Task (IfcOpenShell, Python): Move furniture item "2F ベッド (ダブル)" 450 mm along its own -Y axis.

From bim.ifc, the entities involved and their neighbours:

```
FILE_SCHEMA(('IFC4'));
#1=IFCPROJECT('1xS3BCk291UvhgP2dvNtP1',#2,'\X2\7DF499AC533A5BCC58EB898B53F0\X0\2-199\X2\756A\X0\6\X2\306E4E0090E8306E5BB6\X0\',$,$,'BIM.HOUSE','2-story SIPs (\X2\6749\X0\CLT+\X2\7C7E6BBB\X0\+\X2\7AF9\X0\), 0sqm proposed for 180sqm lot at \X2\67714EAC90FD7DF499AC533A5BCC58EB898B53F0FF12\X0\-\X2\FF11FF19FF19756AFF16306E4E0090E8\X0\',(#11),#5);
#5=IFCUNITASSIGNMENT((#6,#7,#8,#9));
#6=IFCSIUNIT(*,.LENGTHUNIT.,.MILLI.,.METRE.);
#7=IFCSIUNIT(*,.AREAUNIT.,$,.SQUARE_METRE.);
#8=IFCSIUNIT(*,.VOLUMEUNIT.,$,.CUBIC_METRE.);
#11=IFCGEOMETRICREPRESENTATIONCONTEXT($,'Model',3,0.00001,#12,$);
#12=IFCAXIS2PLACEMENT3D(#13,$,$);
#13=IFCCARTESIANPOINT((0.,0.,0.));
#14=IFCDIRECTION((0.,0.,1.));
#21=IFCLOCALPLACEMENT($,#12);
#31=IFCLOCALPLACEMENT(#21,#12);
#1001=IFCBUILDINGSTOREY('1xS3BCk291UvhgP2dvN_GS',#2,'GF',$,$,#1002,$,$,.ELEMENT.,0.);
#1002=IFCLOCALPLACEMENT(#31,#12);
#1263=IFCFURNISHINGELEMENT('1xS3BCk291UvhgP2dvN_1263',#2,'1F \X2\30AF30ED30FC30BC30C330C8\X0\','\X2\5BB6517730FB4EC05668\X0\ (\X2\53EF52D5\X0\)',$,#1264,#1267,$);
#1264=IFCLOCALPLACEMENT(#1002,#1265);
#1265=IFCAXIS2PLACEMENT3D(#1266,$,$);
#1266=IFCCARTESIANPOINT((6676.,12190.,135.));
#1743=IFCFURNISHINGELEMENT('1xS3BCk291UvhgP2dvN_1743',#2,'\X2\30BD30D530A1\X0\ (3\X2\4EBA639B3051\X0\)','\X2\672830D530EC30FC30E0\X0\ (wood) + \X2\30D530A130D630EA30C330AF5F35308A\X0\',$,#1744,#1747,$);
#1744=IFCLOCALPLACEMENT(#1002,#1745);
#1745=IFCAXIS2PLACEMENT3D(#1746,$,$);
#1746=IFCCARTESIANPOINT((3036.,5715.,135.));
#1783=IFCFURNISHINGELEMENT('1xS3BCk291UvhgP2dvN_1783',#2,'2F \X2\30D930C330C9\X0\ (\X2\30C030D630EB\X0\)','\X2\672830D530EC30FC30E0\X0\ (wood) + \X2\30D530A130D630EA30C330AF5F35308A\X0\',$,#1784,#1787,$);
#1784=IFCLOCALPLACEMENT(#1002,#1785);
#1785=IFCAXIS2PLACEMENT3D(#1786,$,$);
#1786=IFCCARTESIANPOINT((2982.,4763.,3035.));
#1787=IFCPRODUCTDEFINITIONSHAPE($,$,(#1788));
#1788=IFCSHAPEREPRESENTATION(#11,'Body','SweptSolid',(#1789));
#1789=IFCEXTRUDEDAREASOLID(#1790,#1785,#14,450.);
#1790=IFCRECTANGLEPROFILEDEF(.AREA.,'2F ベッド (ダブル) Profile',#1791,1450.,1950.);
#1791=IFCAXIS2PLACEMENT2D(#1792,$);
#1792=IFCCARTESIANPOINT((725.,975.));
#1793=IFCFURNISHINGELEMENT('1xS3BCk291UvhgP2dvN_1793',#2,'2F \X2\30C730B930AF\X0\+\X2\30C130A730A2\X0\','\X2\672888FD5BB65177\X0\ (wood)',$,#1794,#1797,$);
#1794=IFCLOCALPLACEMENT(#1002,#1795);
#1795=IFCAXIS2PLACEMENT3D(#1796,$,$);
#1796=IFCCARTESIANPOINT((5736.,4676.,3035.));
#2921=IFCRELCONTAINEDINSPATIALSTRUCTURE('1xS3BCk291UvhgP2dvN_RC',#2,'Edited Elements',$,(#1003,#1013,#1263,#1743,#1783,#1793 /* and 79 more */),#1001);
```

```python
import ifcopenshell
import ifcopenshell.api.geometry
import ifcopenshell.util.placement

model = ifcopenshell.open("bim.ifc")

item = model.by_guid("1xS3BCk291UvhgP2dvN_1783")
matrix = ifcopenshell.util.placement.get_local_placement(item.ObjectPlacement)
matrix[:3, 3] -= matrix[:3, 1] * 450.0
ifcopenshell.api.geometry.edit_object_placement(model, product=item, matrix=matrix, is_si=False)

print(ifcopenshell.util.placement.get_local_placement(item.ObjectPlacement).round(3) + 0.0)

model.write("bim-out.ifc")
```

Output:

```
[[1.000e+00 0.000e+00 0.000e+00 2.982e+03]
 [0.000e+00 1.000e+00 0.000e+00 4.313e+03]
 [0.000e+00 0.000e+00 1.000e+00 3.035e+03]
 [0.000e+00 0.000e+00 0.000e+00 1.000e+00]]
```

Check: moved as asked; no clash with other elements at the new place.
